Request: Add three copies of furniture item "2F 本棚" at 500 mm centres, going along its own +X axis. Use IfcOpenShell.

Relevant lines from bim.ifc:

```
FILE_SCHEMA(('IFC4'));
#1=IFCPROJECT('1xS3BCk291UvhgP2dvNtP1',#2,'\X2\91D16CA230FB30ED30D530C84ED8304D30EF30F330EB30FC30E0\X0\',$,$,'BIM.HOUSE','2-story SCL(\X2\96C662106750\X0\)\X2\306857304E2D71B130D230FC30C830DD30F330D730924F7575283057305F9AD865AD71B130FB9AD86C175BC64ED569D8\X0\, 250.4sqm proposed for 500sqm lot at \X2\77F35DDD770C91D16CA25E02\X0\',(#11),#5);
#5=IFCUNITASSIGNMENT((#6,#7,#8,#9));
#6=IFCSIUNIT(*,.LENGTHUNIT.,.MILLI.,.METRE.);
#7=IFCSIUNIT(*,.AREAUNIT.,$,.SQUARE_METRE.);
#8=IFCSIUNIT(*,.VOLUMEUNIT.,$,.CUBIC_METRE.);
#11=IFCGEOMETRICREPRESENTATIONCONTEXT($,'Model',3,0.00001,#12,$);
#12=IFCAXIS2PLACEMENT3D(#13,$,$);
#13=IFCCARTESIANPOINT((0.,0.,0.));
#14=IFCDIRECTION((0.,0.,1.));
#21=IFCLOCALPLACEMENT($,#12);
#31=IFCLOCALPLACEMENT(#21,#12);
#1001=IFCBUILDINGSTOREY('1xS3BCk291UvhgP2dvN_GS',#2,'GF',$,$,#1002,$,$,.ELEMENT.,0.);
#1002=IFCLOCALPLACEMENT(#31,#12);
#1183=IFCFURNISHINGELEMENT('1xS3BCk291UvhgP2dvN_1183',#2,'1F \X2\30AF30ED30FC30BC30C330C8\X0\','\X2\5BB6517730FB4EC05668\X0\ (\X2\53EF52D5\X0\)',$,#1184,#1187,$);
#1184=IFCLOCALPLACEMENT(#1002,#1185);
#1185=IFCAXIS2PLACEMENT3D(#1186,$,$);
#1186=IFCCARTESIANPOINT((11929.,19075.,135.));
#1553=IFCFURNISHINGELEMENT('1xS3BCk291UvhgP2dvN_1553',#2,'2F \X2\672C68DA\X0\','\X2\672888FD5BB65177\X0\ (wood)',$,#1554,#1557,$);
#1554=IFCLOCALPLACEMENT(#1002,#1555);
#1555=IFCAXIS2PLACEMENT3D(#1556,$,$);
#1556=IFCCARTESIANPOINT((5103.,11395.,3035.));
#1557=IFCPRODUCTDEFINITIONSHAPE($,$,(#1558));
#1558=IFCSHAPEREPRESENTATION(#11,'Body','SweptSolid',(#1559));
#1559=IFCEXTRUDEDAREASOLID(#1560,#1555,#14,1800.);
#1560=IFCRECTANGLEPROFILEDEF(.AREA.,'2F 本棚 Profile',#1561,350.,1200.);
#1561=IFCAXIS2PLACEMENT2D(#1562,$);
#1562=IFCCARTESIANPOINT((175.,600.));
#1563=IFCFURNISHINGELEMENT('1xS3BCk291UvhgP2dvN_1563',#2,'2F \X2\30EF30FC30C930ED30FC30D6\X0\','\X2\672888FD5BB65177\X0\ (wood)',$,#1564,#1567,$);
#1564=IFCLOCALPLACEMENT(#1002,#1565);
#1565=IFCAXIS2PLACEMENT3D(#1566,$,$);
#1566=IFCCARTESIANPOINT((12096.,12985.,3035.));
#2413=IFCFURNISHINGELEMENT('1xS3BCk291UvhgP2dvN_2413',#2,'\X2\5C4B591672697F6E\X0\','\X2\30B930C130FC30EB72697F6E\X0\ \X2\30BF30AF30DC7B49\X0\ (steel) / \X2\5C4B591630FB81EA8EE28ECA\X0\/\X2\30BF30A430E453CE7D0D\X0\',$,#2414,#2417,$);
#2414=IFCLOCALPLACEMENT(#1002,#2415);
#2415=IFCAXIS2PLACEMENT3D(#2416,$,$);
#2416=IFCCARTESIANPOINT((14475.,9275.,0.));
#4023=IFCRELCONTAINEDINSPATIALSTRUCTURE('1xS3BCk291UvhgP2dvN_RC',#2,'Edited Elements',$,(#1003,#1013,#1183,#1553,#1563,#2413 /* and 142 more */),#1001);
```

```python
import ifcopenshell
import ifcopenshell.api.geometry
import ifcopenshell.api.root
import ifcopenshell.util.element
import ifcopenshell.util.placement
import ifcopenshell.util.unit

model = ifcopenshell.open("bim.ifc")
unit_scale = ifcopenshell.util.unit.calculate_unit_scale(model)


def reuse_history(source, copy):
    """copy_class also copies each property set's owner history, people and application; keep the originals."""
    for rel in copy.IsDefinedBy:
        if rel.is_a("IfcRelDefinesByProperties") and (history := rel.RelatingPropertyDefinition.OwnerHistory):
            rel.RelatingPropertyDefinition.OwnerHistory = source.OwnerHistory
            ifcopenshell.util.element.remove_deep2(model, history)


source = model.by_id(1553)
base = ifcopenshell.util.placement.get_local_placement(source.ObjectPlacement)
step = base[:3, 0] * 0.5 / unit_scale

for i in range(1, 4):
    copy = ifcopenshell.api.root.copy_class(model, product=source)
    copy.Representation = ifcopenshell.util.element.copy_deep(
        model, source.Representation, exclude=["IfcGeometricRepresentationContext", "IfcRepresentationMap"]
    )
    reuse_history(source, copy)
    matrix = base.copy()
    matrix[:3, 3] += i * step
    print("added at", matrix[:3, 3].round(3) + 0.0)
    ifcopenshell.api.geometry.edit_object_placement(model, product=copy, matrix=matrix, is_si=False)

model.write("bim_v2.ifc")
```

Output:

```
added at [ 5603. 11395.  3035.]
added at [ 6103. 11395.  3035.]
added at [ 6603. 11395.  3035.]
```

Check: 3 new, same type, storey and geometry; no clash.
